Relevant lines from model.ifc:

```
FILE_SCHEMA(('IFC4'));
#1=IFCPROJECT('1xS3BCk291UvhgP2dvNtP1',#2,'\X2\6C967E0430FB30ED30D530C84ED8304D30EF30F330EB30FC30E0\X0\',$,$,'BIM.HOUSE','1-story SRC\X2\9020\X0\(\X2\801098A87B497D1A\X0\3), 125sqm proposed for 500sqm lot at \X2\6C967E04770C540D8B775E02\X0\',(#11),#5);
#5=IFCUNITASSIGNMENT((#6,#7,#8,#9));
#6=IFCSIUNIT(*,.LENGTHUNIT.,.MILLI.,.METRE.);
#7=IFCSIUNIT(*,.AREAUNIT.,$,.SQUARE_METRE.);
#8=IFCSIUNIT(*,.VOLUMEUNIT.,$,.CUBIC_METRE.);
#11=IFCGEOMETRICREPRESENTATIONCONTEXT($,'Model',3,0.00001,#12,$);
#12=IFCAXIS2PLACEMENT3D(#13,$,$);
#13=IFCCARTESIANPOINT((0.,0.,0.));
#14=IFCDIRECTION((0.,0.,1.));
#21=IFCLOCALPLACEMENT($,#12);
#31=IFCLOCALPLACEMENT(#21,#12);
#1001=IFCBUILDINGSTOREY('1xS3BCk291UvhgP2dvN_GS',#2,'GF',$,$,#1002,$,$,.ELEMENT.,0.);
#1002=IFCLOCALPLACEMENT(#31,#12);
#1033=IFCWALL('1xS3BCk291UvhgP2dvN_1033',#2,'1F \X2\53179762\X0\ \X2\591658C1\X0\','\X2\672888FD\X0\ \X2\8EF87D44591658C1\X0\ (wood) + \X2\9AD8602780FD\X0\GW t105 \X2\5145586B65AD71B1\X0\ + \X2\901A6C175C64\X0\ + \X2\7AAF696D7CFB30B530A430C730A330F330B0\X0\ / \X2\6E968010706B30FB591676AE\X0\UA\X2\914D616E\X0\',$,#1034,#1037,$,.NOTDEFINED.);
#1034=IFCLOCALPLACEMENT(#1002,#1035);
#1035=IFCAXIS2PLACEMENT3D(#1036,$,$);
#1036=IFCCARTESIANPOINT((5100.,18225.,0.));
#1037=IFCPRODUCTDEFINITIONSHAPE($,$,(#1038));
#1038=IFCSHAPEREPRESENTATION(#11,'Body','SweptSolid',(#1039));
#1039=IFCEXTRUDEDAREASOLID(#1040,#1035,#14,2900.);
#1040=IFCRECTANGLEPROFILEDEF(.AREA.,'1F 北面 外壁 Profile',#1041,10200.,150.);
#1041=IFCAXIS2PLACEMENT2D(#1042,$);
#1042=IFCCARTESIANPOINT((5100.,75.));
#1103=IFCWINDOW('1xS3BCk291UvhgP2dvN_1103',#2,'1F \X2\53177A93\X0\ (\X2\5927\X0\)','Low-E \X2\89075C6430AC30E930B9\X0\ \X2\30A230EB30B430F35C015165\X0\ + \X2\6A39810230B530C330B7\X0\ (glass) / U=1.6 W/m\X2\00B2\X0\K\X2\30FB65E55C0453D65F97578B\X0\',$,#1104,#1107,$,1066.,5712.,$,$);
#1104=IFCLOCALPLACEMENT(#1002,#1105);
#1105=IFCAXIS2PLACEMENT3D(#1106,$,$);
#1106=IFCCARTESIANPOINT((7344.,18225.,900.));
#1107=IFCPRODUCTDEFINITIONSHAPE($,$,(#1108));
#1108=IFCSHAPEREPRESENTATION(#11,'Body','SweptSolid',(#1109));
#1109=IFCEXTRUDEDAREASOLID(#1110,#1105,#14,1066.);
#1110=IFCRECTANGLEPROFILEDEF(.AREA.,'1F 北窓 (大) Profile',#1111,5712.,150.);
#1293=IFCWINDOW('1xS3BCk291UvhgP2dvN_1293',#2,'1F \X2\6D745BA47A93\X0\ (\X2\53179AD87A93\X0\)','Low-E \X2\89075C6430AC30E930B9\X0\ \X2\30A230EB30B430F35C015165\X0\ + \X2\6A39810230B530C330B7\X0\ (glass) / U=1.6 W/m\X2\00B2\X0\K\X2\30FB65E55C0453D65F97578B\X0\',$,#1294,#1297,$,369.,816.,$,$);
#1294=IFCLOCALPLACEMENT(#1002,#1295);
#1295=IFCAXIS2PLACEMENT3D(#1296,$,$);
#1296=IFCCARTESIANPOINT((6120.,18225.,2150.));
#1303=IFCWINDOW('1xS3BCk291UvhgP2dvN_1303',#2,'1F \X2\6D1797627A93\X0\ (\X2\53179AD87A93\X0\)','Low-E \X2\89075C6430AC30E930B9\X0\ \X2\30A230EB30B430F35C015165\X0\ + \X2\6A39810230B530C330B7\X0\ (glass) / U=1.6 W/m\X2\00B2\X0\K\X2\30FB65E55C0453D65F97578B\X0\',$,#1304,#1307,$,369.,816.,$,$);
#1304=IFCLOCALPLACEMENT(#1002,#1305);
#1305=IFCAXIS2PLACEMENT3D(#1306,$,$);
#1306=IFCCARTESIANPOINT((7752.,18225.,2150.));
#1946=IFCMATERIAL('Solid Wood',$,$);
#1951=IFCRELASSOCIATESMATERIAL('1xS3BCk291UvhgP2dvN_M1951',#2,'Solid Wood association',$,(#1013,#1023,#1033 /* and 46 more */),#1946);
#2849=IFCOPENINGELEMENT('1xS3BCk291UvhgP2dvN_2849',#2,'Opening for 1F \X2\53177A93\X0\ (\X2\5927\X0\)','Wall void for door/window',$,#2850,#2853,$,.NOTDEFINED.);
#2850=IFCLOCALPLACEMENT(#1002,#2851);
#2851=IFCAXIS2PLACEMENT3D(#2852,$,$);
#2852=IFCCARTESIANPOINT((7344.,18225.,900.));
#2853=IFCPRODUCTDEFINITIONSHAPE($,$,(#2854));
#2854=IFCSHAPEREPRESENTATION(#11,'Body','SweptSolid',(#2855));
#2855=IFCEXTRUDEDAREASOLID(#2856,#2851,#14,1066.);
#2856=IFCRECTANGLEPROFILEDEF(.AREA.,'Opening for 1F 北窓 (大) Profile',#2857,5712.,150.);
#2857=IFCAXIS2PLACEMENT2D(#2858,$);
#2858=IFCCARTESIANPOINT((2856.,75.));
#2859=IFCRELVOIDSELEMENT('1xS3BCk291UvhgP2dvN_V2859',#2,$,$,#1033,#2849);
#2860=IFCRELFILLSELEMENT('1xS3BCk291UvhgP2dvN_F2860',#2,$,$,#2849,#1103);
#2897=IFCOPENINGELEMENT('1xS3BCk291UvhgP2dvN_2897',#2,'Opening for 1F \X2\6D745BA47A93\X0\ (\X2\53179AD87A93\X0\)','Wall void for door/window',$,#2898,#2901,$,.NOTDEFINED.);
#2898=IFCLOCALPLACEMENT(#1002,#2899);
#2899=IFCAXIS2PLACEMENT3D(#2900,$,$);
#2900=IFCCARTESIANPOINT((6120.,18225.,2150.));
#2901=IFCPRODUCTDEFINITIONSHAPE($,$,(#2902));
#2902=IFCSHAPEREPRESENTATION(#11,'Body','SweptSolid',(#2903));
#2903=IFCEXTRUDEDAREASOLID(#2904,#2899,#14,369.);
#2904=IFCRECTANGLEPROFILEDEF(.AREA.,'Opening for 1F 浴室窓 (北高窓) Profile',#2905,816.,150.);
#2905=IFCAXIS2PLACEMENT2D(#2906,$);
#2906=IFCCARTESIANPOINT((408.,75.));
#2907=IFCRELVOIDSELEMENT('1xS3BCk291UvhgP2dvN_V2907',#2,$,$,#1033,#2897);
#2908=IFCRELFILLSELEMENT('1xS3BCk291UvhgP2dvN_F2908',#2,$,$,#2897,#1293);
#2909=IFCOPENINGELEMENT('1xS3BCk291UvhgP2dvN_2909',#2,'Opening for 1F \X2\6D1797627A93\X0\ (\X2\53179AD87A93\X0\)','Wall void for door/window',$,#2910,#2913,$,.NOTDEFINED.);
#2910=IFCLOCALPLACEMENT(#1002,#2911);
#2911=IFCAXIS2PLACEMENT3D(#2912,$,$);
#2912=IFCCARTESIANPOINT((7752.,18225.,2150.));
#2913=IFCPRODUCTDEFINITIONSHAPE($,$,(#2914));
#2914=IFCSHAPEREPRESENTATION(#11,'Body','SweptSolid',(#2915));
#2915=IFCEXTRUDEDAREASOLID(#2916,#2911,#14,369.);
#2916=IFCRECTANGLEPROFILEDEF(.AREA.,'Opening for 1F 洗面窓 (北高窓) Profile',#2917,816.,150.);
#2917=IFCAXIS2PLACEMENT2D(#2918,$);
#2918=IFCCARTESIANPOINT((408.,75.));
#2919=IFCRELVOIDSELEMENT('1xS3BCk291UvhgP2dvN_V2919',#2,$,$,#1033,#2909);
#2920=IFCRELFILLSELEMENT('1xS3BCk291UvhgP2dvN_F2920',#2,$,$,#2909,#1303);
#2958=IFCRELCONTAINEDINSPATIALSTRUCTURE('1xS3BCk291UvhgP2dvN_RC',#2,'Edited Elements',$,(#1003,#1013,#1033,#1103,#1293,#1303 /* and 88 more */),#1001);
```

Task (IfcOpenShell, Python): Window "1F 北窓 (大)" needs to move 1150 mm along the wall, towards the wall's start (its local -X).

```python
import ifcopenshell
import ifcopenshell.api.geometry
import ifcopenshell.util.placement
import ifcopenshell.util.unit

model = ifcopenshell.open("model.ifc")
unit_scale = ifcopenshell.util.unit.calculate_unit_scale(model)

window = model.by_id(1103)
opening = window.FillsVoids[0].RelatingOpeningElement
wall = opening.VoidsElements[0].RelatingBuildingElement

wall_matrix = ifcopenshell.util.placement.get_local_placement(wall.ObjectPlacement)
shift = wall_matrix[:3, 0] * -1.15 / unit_scale
before = ifcopenshell.util.placement.get_local_placement(window.ObjectPlacement)[:3, 3].copy()

# The window is not placed relative to its opening, so move both.
for product in (opening, window):
    matrix = ifcopenshell.util.placement.get_local_placement(product.ObjectPlacement)
    matrix[:3, 3] += shift
    ifcopenshell.api.geometry.edit_object_placement(model, product=product, matrix=matrix, is_si=False)

after = ifcopenshell.util.placement.get_local_placement(window.ObjectPlacement)[:3, 3]
print("window moved by", (after - before).round(3) + 0.0)

model.write("model_v2.ifc")
```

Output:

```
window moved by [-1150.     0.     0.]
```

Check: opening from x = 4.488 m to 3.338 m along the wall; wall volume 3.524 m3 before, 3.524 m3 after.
